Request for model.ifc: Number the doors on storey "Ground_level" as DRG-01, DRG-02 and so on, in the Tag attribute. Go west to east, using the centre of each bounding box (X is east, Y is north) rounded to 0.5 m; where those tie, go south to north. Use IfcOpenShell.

First a look at what the model holds.

```python
import ifcopenshell
import ifcopenshell.util.element
import ifcopenshell.util.placement

model = ifcopenshell.open("model.ifc")
print(model.schema)
storey = next(s for s in model.by_type("IfcBuildingStorey") if s.Name == "Ground_level")
doors = [e for e in ifcopenshell.util.element.get_decomposition(storey) if e.is_a("IfcDoor")]
for e in sorted(doors, key=lambda e: e.id()):
    origin = ifcopenshell.util.placement.get_local_placement(e.ObjectPlacement)[:3, 3]
    print(e.id(), e.Tag, e.Name, origin.round(2) + 0.0, sep=" | ")
```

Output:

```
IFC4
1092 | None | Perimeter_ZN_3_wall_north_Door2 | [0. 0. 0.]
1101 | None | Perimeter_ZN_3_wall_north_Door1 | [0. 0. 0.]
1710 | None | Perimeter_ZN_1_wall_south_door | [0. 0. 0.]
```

```python
import ifcopenshell
import ifcopenshell.geom
import ifcopenshell.util.element
import ifcopenshell.util.shape

model = ifcopenshell.open("model.ifc")
settings = ifcopenshell.geom.settings()
settings.set("use-world-coords", True)


def centre(element):
    shape = ifcopenshell.geom.create_shape(settings, element)
    return ifcopenshell.util.shape.get_bbox_centroid(shape.geometry)


storey = next(s for s in model.by_type("IfcBuildingStorey") if s.Name == "Ground_level")
doors = [e for e in ifcopenshell.util.element.get_decomposition(storey) if e.is_a("IfcDoor")]

# Insertion points can sit at a corner or the storey origin, so sort by the geometry (in metres).
centres = {e: centre(e) for e in doors}
doors.sort(key=lambda e: (round(centres[e][0] / 0.5), centres[e][1]))

for i, e in enumerate(doors, start=1):
    number = f"DRG-{i:02d}"
    e.Tag = number
    print(e.id(), number)

model.write("model_edited.ifc")
```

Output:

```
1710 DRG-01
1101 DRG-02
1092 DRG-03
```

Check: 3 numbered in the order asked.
